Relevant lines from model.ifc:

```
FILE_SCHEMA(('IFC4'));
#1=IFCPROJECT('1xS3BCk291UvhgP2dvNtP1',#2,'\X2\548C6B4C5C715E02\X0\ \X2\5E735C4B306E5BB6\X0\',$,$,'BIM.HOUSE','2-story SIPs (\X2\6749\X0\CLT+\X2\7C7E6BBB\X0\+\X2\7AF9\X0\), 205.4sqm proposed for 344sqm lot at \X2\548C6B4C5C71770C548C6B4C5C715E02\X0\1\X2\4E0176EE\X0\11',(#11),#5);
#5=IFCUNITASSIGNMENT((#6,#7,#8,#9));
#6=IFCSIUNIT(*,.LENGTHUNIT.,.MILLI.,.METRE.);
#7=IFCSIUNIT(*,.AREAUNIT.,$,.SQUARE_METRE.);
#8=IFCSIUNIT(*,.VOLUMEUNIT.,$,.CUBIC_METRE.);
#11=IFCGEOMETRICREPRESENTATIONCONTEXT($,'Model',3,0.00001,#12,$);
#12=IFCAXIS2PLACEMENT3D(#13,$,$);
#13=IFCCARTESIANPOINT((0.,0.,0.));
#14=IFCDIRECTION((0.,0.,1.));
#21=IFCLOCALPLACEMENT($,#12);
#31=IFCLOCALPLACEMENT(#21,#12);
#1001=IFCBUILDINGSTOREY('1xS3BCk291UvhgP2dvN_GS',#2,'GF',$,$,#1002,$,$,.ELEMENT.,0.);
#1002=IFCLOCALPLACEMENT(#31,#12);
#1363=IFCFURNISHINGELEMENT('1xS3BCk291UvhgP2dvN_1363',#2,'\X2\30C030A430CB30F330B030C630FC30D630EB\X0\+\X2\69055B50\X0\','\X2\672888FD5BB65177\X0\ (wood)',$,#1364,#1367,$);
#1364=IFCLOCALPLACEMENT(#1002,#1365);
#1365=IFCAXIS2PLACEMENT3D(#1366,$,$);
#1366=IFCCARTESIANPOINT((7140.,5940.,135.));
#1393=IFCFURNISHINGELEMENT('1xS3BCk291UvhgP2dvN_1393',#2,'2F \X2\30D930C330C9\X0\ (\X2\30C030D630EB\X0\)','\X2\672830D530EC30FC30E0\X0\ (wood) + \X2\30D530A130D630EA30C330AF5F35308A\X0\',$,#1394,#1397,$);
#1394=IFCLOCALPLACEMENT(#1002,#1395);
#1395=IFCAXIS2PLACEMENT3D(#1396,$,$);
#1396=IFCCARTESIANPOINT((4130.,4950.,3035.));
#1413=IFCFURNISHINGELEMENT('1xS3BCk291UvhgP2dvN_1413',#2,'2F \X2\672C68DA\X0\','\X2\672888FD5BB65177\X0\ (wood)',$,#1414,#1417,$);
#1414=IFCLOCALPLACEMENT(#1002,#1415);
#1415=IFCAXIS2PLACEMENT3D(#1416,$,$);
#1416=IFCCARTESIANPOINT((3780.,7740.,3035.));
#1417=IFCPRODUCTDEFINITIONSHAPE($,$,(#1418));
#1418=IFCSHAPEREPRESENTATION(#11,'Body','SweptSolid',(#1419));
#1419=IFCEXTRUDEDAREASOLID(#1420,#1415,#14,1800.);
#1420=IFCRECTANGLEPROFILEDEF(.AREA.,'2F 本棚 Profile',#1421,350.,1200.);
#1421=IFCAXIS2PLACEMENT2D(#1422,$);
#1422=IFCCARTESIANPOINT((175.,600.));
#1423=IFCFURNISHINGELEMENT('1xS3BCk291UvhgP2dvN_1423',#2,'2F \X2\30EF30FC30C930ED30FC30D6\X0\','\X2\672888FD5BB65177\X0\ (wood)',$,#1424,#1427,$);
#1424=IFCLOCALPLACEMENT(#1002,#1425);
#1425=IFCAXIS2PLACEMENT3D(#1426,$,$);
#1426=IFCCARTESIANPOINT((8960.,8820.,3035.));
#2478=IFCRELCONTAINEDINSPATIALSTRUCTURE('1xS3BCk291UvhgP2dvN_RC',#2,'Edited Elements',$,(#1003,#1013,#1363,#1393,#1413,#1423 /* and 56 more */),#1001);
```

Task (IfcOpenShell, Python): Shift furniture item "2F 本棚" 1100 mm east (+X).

```python
import ifcopenshell
import ifcopenshell.api.geometry
import ifcopenshell.util.placement
import ifcopenshell.util.unit

model = ifcopenshell.open("model.ifc")
unit_scale = ifcopenshell.util.unit.calculate_unit_scale(model)

item = model.by_guid("1xS3BCk291UvhgP2dvN_1413")
matrix = ifcopenshell.util.placement.get_local_placement(item.ObjectPlacement)
matrix[0, 3] += 1.1 / unit_scale
ifcopenshell.api.geometry.edit_object_placement(model, product=item, matrix=matrix, is_si=False)

print(ifcopenshell.util.placement.get_local_placement(item.ObjectPlacement).round(3) + 0.0)

model.write("model_updated.ifc")
```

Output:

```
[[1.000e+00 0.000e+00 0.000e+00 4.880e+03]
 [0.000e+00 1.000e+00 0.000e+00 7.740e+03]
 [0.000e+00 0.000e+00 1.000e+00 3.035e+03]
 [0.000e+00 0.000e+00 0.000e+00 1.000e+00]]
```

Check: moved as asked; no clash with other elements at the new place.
